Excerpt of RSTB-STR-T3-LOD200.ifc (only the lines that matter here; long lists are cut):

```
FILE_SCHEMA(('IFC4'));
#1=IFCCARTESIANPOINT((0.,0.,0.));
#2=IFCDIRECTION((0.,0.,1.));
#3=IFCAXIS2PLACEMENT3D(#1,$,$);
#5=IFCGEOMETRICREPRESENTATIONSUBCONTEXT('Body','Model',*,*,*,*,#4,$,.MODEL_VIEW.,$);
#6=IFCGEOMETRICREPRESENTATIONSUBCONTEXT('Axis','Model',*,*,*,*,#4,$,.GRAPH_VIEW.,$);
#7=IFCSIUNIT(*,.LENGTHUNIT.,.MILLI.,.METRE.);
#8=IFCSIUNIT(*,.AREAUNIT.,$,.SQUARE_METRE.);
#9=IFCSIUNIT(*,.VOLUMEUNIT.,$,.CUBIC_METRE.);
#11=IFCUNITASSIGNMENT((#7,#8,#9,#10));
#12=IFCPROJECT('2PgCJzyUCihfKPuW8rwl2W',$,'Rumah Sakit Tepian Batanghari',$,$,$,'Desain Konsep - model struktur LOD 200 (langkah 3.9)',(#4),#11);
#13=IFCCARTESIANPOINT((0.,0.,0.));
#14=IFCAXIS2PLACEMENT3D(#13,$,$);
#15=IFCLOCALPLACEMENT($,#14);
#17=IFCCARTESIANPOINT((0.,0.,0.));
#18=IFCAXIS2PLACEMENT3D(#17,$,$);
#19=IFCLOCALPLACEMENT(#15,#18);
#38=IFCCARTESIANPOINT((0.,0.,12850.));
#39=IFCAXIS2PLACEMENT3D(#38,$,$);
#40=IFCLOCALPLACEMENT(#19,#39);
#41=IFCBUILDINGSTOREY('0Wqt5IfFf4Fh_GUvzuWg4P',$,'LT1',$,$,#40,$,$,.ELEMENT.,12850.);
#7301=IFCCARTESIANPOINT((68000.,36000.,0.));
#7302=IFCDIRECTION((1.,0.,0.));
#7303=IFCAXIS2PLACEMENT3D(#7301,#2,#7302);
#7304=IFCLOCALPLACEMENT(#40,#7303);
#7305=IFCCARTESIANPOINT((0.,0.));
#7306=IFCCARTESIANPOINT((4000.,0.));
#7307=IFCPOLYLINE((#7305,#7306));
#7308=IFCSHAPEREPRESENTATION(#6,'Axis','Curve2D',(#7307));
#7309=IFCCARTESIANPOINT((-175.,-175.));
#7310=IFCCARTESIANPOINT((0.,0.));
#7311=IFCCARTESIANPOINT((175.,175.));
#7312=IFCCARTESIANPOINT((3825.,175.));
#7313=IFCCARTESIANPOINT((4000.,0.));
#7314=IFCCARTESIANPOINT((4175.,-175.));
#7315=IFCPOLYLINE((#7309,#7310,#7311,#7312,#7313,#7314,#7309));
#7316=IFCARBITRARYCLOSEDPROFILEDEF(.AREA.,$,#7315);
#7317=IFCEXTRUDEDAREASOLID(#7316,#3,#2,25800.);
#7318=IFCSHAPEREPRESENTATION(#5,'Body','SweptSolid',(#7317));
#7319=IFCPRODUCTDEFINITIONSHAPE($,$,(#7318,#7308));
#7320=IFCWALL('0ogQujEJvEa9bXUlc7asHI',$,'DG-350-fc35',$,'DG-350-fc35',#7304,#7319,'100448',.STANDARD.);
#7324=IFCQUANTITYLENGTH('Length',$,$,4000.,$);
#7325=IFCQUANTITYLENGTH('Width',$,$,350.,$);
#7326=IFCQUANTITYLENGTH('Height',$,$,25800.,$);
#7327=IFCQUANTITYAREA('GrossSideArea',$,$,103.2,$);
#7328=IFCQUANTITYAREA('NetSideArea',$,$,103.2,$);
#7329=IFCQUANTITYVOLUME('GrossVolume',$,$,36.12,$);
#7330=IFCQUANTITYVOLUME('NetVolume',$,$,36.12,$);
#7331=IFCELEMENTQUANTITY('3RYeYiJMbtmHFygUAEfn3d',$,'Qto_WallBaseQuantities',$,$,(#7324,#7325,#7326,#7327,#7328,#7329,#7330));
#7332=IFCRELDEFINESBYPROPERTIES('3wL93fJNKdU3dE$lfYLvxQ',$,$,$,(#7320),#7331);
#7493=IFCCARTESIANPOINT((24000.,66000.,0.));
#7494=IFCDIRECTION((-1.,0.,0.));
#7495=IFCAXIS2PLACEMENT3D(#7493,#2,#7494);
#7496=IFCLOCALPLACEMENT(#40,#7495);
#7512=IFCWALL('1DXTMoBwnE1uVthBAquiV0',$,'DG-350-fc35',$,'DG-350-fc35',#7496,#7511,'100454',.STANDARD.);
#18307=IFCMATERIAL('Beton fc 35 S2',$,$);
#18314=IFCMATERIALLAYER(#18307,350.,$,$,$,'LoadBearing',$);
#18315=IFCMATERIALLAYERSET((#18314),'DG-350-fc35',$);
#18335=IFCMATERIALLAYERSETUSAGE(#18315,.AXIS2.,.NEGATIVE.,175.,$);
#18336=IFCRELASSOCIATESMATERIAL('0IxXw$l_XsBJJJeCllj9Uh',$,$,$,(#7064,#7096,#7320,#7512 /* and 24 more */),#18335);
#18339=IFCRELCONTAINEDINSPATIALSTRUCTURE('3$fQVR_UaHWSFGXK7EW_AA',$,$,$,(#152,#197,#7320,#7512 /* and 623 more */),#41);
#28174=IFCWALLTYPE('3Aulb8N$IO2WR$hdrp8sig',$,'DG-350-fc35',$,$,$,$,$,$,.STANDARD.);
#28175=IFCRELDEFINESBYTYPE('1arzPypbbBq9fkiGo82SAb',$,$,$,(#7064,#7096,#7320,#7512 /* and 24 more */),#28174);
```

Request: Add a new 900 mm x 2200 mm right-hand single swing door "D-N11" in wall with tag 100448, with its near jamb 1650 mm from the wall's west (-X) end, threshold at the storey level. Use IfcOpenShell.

```python
import numpy as np
import ifcopenshell
import ifcopenshell.api.feature
import ifcopenshell.api.geometry
import ifcopenshell.api.pset
import ifcopenshell.api.root
import ifcopenshell.api.spatial
import ifcopenshell.geom
import ifcopenshell.util.element
import ifcopenshell.util.placement
import ifcopenshell.util.representation
import ifcopenshell.util.shape
import ifcopenshell.util.unit

model = ifcopenshell.open("RSTB-STR-T3-LOD200.ifc")
unit_scale = ifcopenshell.util.unit.calculate_unit_scale(model)
area_scale = ifcopenshell.util.unit.calculate_unit_scale(model, "AREAUNIT")
volume_scale = ifcopenshell.util.unit.calculate_unit_scale(model, "VOLUMEUNIT")
settings = ifcopenshell.geom.settings()


def volume(element):
    """Net volume in cubic metres, openings subtracted."""
    shape = ifcopenshell.geom.create_shape(settings, element)
    return ifcopenshell.util.shape.get_volume(shape.geometry)


wall = model.by_guid("0ogQujEJvEa9bXUlc7asHI")
storey = ifcopenshell.util.element.get_container(wall, ifc_class="IfcBuildingStorey")
context = ifcopenshell.util.representation.get_context(model, "Model", "Body", "MODEL_VIEW")
before = volume(wall)

width, height, from_end, sill = 0.9, 2.2, 1.65, 0.0  # metres

# The wall runs along its own X axis, and the end named is its -X end.
wall_shape = ifcopenshell.geom.create_shape(settings, wall)
x, y, z = ifcopenshell.util.shape.get_vertices(wall_shape.geometry).T
start = x.min() + from_end
face, thickness = float(y.min()), float(y.max() - y.min())
wall_matrix = ifcopenshell.util.placement.get_local_placement(wall.ObjectPlacement)
level = ifcopenshell.util.placement.get_local_placement(storey.ObjectPlacement)[2, 3]


def in_wall(x, y):
    """Placement at x, y metres in the wall's axes, at sill height."""
    matrix = wall_matrix.copy()
    matrix[:, 3] = wall_matrix @ np.array([x / unit_scale, y / unit_scale, 0.0, 1.0])
    matrix[2, 3] = level + sill / unit_scale
    return matrix


# Opening: a box that overshoots both wall faces by 50 mm.
opening = ifcopenshell.api.root.create_entity(model, ifc_class="IfcOpeningElement", predefined_type="OPENING")
box = ifcopenshell.api.geometry.add_wall_representation(
    model, context=context, length=width, height=height, thickness=thickness + 0.1
)
ifcopenshell.api.geometry.assign_representation(model, product=opening, representation=box)
ifcopenshell.api.geometry.edit_object_placement(model, product=opening, matrix=in_wall(start, face - 0.05), is_si=False)
ifcopenshell.api.feature.add_feature(model, feature=opening, element=wall)

door = ifcopenshell.api.root.create_entity(model, ifc_class="IfcDoor", name="D-N11", predefined_type="DOOR")
door.OverallWidth, door.OverallHeight = width / unit_scale, height / unit_scale
door.OperationType = "SINGLE_SWING_RIGHT"
body = ifcopenshell.api.geometry.add_door_representation(
    model,
    context=context,
    overall_width=door.OverallWidth,
    overall_height=door.OverallHeight,
    operation_type="SINGLE_SWING_RIGHT",
    lining_properties={"LiningDepth": thickness / unit_scale, "ThresholdDepth": thickness / unit_scale},
)
ifcopenshell.api.geometry.assign_representation(model, product=door, representation=body)
ifcopenshell.api.spatial.assign_container(model, products=[door], relating_structure=storey)
ifcopenshell.api.feature.add_filling(model, opening=opening, element=door)

# The lining spans the wall, so the door starts at the wall face.
ifcopenshell.api.geometry.edit_object_placement(model, product=door, matrix=in_wall(start, face), is_si=False)

after = volume(wall)

# Update the wall's stored quantities.
qto = model.by_id(ifcopenshell.util.element.get_pset(wall, "Qto_WallBaseQuantities", should_inherit=False)["id"])
ifcopenshell.api.pset.edit_qto(model, qto=qto, properties={
    "NetSideArea": after / thickness / area_scale,
    "NetVolume": after / volume_scale,
})

print(f"wall volume {before:.3f} -> {after:.3f} m3")

model.write("RSTB-STR-T3-LOD200_v2.ifc")
```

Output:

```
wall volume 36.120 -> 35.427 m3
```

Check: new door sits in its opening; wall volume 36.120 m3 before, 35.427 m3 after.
